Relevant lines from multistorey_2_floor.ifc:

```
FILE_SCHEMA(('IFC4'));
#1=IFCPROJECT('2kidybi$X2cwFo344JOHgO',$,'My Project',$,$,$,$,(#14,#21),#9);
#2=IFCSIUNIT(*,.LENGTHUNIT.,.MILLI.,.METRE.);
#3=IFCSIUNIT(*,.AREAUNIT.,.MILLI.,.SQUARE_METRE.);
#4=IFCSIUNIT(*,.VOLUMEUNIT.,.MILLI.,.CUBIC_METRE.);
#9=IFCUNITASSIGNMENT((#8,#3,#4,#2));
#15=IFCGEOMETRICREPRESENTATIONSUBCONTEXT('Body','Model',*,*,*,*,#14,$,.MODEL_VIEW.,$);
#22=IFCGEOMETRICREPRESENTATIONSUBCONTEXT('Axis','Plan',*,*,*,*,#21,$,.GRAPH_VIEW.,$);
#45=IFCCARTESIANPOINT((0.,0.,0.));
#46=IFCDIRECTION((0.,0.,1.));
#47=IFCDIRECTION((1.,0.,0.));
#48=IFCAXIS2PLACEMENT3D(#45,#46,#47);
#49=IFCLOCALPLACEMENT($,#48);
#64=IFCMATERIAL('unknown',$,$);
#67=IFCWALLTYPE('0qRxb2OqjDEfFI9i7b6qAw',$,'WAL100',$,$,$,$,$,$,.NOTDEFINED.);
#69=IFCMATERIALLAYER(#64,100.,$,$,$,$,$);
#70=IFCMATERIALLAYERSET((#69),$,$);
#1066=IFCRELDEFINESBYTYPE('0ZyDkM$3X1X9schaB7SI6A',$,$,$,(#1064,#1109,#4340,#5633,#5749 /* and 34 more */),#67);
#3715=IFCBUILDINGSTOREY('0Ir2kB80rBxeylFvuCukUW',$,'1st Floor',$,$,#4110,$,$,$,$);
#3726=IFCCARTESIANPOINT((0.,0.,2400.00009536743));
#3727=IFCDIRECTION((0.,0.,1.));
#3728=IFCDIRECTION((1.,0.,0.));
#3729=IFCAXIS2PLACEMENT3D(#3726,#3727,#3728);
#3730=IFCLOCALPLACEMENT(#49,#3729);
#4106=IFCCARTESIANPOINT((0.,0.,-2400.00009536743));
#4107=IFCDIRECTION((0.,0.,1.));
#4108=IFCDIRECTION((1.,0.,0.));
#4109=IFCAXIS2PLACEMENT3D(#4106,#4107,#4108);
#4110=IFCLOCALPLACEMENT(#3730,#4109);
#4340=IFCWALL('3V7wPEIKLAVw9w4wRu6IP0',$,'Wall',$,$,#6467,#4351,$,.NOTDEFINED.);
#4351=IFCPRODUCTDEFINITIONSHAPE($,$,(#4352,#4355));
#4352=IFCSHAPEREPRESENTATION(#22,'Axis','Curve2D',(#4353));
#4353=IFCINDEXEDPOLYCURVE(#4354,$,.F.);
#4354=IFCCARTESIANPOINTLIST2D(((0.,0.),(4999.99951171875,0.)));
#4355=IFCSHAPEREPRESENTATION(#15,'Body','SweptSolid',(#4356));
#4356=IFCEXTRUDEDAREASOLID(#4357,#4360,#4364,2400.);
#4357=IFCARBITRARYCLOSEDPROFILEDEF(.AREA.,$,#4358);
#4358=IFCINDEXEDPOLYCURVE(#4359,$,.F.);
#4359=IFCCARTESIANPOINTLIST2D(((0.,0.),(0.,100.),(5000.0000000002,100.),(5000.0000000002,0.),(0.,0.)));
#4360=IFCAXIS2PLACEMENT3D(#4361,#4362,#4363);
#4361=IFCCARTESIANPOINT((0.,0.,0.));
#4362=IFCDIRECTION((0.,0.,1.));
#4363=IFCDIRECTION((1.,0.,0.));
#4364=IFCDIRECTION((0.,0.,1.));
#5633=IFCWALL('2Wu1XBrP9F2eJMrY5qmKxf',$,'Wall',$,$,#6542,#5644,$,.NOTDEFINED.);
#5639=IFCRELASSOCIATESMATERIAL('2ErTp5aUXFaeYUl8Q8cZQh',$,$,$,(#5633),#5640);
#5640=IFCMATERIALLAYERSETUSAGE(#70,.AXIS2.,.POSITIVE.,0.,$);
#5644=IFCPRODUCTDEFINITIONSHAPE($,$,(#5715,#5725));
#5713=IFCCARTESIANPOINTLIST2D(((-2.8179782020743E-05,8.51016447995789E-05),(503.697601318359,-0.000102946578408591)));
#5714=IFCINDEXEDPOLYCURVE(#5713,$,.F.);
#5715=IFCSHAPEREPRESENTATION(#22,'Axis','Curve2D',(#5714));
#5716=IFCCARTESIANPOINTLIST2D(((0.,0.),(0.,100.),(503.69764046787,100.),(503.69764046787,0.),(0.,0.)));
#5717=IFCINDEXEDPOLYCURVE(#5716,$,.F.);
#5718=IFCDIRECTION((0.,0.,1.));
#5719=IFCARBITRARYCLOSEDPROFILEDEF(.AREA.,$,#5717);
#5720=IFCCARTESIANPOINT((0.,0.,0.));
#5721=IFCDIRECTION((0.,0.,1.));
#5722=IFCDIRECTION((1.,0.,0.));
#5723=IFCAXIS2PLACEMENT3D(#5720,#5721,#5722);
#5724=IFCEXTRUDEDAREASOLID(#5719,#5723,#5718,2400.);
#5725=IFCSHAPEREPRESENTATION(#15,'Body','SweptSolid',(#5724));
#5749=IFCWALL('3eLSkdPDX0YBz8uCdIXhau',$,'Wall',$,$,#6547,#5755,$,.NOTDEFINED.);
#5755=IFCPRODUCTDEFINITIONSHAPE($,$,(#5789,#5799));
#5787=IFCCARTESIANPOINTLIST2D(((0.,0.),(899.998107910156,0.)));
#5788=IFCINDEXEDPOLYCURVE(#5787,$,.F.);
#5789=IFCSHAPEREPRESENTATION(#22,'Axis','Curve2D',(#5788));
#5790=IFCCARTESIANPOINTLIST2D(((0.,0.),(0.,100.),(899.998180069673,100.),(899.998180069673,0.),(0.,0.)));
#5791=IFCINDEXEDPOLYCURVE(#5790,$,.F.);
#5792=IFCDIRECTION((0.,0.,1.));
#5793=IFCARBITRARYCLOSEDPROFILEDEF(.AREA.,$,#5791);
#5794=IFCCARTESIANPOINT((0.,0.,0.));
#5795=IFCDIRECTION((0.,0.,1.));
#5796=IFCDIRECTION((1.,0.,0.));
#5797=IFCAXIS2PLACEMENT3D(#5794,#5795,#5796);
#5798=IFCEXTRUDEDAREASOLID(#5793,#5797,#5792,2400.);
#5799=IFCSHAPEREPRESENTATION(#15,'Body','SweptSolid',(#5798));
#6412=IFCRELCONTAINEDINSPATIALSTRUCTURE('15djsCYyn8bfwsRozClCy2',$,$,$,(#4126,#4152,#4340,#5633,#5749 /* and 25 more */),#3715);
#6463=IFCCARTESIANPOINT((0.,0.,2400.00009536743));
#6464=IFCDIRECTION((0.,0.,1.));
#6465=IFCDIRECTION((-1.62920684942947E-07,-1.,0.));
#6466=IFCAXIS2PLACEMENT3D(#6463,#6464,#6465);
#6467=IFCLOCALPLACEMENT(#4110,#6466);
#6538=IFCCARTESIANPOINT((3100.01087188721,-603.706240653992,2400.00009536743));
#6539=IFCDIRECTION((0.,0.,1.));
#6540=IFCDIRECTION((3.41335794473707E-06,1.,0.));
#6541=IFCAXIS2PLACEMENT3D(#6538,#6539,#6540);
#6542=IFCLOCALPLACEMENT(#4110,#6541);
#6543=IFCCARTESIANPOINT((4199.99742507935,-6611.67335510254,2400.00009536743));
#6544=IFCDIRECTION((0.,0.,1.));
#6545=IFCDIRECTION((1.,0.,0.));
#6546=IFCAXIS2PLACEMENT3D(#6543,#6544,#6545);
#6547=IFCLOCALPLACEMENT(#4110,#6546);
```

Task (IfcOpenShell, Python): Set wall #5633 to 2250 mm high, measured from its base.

```python
import ifcopenshell
import ifcopenshell.geom
import ifcopenshell.util.representation
import ifcopenshell.util.shape

model = ifcopenshell.open("multistorey_2_floor.ifc")
settings = ifcopenshell.geom.settings()


def volume(element):
    """Net volume in cubic metres, openings subtracted."""
    shape = ifcopenshell.geom.create_shape(settings, element)
    return ifcopenshell.util.shape.get_volume(shape.geometry)


wall = model.by_id(5633)
before = volume(wall)

body = ifcopenshell.util.representation.get_representation(wall, "Model", "Body")
solid = body.Items[0]
old_height = solid.Depth
solid.Depth = 2250.0
after = volume(wall)

print(f"height {old_height:g} -> {solid.Depth:g}, volume {before:.3f} -> {after:.3f} m3")

model.write("multistorey_2_floor_v2.ifc")
```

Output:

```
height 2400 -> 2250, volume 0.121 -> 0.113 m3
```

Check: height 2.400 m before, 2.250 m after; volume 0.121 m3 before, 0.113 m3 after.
